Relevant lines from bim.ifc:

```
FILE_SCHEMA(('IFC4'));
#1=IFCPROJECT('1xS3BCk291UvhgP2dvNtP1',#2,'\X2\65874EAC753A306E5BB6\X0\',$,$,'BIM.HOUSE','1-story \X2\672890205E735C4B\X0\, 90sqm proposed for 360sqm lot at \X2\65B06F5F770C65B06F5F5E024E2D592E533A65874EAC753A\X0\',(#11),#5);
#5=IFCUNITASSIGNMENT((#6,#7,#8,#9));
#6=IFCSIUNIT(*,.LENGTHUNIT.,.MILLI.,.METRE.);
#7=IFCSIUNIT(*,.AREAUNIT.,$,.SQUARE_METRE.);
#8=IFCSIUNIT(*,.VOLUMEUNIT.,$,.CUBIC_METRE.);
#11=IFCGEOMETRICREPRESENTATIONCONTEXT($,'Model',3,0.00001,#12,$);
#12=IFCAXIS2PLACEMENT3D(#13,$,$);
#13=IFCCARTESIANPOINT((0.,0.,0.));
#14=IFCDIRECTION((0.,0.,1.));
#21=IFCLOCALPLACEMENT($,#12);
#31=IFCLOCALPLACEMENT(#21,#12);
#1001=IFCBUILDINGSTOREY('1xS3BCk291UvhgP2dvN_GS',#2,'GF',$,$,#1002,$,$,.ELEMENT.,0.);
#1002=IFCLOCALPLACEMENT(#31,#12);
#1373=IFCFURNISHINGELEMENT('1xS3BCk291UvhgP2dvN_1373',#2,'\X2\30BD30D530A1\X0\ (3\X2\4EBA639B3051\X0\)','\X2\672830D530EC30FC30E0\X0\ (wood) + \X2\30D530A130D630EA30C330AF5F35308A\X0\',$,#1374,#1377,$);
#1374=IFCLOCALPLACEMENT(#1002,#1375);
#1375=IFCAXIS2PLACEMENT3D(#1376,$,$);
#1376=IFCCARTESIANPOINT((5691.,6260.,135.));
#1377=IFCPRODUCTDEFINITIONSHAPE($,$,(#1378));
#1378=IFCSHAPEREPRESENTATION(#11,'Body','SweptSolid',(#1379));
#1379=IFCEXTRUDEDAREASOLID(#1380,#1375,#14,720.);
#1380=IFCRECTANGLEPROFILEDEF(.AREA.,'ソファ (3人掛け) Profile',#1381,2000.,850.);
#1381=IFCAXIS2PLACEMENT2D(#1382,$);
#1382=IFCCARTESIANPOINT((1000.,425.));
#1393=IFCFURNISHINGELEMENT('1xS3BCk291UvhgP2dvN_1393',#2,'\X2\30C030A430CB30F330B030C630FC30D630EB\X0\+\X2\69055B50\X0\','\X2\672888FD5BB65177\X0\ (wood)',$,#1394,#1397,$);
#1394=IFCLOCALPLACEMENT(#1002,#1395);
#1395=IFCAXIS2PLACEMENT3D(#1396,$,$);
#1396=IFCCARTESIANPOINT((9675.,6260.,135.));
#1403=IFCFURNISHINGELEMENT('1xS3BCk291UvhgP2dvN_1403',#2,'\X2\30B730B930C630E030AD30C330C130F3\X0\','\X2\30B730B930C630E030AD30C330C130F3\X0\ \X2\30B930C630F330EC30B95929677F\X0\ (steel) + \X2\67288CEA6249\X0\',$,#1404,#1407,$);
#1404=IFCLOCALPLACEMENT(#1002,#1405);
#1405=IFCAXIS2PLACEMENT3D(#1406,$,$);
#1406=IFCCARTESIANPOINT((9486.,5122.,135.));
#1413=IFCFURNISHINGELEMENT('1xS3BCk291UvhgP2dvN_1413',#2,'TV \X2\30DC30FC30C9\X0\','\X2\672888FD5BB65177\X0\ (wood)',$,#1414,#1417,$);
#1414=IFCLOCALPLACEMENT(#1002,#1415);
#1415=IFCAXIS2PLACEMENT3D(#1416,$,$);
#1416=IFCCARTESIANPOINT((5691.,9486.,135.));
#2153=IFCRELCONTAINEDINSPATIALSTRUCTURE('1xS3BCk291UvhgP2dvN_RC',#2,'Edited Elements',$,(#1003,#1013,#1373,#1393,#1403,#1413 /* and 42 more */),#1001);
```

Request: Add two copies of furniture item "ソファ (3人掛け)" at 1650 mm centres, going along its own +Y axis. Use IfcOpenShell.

```python
import ifcopenshell
import ifcopenshell.api.geometry
import ifcopenshell.api.root
import ifcopenshell.util.element
import ifcopenshell.util.placement
import ifcopenshell.util.unit

model = ifcopenshell.open("bim.ifc")
unit_scale = ifcopenshell.util.unit.calculate_unit_scale(model)


def reuse_history(source, copy):
    """copy_class also copies each property set's owner history, people and application; keep the originals."""
    for rel in copy.IsDefinedBy:
        if rel.is_a("IfcRelDefinesByProperties") and (history := rel.RelatingPropertyDefinition.OwnerHistory):
            rel.RelatingPropertyDefinition.OwnerHistory = source.OwnerHistory
            ifcopenshell.util.element.remove_deep2(model, history)


source = model.by_guid("1xS3BCk291UvhgP2dvN_1373")
base = ifcopenshell.util.placement.get_local_placement(source.ObjectPlacement)
step = base[:3, 1] * 1.65 / unit_scale

for i in range(1, 3):
    copy = ifcopenshell.api.root.copy_class(model, product=source)
    copy.Representation = ifcopenshell.util.element.copy_deep(
        model, source.Representation, exclude=["IfcGeometricRepresentationContext", "IfcRepresentationMap"]
    )
    reuse_history(source, copy)
    matrix = base.copy()
    matrix[:3, 3] += i * step
    print("added at", matrix[:3, 3].round(3) + 0.0)
    ifcopenshell.api.geometry.edit_object_placement(model, product=copy, matrix=matrix, is_si=False)

model.write("bim_edited.ifc")
```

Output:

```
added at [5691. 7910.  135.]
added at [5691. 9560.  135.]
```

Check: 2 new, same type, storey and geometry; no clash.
